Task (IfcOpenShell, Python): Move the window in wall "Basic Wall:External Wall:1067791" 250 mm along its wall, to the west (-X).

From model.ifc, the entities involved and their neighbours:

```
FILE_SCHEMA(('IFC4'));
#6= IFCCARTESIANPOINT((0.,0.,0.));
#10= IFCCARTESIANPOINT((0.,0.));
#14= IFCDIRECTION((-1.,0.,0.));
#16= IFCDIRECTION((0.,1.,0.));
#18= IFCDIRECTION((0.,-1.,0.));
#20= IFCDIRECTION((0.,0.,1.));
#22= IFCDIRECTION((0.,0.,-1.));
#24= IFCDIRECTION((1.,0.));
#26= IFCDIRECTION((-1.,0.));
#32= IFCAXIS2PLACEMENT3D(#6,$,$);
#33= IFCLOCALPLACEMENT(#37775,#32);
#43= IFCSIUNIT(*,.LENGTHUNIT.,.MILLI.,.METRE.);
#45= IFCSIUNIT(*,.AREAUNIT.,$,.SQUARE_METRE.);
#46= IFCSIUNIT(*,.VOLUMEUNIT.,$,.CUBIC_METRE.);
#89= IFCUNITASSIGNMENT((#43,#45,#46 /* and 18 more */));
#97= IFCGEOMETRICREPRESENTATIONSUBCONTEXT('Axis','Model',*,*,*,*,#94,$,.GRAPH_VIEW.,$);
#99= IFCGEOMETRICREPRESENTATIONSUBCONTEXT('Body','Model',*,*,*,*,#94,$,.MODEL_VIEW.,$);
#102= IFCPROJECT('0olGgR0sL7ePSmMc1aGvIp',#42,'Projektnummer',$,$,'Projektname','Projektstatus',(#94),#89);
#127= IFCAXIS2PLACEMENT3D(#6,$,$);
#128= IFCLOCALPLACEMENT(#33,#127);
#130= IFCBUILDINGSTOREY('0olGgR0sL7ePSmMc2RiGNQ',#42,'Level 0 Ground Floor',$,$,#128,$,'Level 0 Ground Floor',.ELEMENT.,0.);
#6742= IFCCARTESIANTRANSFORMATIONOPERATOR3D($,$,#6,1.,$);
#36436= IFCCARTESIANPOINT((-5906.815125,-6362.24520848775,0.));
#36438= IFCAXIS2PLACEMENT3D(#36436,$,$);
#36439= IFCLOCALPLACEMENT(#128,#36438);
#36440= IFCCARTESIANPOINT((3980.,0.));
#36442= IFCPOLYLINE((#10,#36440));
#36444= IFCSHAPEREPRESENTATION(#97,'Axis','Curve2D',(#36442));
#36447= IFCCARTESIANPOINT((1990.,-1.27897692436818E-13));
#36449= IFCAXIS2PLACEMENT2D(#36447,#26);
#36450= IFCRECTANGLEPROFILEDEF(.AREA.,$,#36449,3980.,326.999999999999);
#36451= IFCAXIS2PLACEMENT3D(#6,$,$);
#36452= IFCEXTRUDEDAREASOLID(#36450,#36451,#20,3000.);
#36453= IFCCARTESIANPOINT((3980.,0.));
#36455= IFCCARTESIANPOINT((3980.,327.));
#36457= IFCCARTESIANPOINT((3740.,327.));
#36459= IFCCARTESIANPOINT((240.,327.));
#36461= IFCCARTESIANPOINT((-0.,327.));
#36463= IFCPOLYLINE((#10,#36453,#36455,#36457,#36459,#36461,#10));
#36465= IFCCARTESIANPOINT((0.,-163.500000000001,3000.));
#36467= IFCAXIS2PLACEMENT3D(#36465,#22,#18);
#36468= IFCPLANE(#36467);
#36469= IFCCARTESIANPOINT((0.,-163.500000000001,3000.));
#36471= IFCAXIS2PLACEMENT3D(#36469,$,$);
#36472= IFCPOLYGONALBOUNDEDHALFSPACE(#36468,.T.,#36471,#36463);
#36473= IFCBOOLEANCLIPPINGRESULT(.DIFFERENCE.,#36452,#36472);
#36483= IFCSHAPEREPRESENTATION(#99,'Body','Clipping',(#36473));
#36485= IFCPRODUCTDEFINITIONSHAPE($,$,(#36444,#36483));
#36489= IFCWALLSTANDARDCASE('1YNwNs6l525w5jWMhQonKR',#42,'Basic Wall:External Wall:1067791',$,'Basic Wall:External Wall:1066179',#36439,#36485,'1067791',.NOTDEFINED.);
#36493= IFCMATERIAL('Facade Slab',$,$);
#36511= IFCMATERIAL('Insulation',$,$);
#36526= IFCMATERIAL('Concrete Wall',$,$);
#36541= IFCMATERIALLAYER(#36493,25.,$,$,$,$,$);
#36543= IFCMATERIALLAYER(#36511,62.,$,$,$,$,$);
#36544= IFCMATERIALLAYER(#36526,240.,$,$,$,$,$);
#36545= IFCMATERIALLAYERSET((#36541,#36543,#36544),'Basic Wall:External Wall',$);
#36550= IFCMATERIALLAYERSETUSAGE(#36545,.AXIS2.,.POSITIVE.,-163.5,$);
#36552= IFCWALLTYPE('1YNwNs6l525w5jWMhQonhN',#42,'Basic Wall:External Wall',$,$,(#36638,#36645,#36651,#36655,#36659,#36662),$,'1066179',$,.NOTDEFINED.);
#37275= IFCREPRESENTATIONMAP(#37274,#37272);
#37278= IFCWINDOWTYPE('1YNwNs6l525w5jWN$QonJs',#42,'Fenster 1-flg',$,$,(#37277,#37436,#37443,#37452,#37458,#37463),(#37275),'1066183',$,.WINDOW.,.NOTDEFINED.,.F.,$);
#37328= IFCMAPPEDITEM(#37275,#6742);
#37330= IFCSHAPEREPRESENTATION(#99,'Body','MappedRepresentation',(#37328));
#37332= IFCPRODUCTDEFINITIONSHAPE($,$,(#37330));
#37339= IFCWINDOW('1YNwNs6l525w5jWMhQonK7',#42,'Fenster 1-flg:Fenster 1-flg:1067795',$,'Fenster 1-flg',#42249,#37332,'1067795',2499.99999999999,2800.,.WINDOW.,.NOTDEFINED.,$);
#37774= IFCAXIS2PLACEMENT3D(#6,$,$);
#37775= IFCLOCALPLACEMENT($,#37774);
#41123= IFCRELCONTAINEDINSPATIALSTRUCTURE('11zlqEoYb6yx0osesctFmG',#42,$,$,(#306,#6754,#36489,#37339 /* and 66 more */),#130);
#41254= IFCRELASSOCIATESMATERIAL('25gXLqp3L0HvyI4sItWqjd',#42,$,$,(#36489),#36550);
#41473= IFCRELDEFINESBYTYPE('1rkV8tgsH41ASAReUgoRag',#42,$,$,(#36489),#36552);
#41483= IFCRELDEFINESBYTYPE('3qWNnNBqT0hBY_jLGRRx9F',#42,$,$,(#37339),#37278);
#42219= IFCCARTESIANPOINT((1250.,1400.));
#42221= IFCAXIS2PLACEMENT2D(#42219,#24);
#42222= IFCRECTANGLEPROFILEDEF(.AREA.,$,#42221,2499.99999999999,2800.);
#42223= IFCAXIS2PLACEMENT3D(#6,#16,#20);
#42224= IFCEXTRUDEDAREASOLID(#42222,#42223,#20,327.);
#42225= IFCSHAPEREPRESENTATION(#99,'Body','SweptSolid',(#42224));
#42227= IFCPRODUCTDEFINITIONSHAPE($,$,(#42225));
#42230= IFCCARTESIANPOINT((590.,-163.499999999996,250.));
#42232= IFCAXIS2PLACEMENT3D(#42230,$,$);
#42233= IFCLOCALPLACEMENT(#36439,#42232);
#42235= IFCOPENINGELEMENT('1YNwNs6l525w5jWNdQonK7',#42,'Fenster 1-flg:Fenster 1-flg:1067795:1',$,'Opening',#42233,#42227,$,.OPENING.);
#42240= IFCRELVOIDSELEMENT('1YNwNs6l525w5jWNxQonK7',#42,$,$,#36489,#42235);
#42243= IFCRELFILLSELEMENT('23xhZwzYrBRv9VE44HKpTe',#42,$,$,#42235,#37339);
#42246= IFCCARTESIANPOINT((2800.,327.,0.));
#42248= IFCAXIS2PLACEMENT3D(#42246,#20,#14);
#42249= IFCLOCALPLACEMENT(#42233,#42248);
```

```python
import ifcopenshell
import ifcopenshell.api.geometry
import ifcopenshell.util.placement

model = ifcopenshell.open("model.ifc")

window = model.by_id(37339)
opening = window.FillsVoids[0].RelatingOpeningElement
wall = opening.VoidsElements[0].RelatingBuildingElement

wall_matrix = ifcopenshell.util.placement.get_local_placement(wall.ObjectPlacement)
shift = wall_matrix[:3, 0] * -250.0
before = ifcopenshell.util.placement.get_local_placement(window.ObjectPlacement)[:3, 3].copy()

# The window is placed relative to its opening, so it follows when the opening moves.
matrix = ifcopenshell.util.placement.get_local_placement(opening.ObjectPlacement)
matrix[:3, 3] += shift
ifcopenshell.api.geometry.edit_object_placement(
    model, product=opening, matrix=matrix, is_si=False, should_transform_children=True
)

after = ifcopenshell.util.placement.get_local_placement(window.ObjectPlacement)[:3, 3]
print("window moved by", (after - before).round(3) + 0.0)

model.write("model_v2.ifc")
```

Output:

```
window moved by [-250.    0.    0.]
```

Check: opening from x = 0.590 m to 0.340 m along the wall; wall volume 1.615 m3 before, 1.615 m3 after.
